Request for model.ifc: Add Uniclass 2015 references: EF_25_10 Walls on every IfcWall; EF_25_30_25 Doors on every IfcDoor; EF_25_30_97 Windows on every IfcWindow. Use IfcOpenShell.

First a look at what the model holds.

```python
import ifcopenshell

model = ifcopenshell.open("model.ifc")
print(model.schema)
print("classifications:", [c.Name for c in model.by_type("IfcClassification")])
for ifc_class in ("IfcDoor", "IfcRoof", "IfcStair", "IfcWall", "IfcWindow"):
    print(ifc_class, len(model.by_type(ifc_class)))
```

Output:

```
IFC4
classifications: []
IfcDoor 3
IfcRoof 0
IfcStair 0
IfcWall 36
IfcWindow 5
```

```python
import ifcopenshell
import ifcopenshell.api.classification

model = ifcopenshell.open("model.ifc")

system = ifcopenshell.api.classification.add_classification(model, classification="Uniclass 2015")

codes = {
    "IfcWall": ("EF_25_10", "Walls"),
    "IfcDoor": ("EF_25_30_25", "Doors"),
    "IfcWindow": ("EF_25_30_97", "Windows"),
}
for ifc_class, (code, name) in codes.items():
    products = model.by_type(ifc_class)
    ifcopenshell.api.classification.add_reference(
        model, products=products, classification=system, identification=code, name=name
    )
    print(code, len(products))

model.write("model_updated.ifc")
```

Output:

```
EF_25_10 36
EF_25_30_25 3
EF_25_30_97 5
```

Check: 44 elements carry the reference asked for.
